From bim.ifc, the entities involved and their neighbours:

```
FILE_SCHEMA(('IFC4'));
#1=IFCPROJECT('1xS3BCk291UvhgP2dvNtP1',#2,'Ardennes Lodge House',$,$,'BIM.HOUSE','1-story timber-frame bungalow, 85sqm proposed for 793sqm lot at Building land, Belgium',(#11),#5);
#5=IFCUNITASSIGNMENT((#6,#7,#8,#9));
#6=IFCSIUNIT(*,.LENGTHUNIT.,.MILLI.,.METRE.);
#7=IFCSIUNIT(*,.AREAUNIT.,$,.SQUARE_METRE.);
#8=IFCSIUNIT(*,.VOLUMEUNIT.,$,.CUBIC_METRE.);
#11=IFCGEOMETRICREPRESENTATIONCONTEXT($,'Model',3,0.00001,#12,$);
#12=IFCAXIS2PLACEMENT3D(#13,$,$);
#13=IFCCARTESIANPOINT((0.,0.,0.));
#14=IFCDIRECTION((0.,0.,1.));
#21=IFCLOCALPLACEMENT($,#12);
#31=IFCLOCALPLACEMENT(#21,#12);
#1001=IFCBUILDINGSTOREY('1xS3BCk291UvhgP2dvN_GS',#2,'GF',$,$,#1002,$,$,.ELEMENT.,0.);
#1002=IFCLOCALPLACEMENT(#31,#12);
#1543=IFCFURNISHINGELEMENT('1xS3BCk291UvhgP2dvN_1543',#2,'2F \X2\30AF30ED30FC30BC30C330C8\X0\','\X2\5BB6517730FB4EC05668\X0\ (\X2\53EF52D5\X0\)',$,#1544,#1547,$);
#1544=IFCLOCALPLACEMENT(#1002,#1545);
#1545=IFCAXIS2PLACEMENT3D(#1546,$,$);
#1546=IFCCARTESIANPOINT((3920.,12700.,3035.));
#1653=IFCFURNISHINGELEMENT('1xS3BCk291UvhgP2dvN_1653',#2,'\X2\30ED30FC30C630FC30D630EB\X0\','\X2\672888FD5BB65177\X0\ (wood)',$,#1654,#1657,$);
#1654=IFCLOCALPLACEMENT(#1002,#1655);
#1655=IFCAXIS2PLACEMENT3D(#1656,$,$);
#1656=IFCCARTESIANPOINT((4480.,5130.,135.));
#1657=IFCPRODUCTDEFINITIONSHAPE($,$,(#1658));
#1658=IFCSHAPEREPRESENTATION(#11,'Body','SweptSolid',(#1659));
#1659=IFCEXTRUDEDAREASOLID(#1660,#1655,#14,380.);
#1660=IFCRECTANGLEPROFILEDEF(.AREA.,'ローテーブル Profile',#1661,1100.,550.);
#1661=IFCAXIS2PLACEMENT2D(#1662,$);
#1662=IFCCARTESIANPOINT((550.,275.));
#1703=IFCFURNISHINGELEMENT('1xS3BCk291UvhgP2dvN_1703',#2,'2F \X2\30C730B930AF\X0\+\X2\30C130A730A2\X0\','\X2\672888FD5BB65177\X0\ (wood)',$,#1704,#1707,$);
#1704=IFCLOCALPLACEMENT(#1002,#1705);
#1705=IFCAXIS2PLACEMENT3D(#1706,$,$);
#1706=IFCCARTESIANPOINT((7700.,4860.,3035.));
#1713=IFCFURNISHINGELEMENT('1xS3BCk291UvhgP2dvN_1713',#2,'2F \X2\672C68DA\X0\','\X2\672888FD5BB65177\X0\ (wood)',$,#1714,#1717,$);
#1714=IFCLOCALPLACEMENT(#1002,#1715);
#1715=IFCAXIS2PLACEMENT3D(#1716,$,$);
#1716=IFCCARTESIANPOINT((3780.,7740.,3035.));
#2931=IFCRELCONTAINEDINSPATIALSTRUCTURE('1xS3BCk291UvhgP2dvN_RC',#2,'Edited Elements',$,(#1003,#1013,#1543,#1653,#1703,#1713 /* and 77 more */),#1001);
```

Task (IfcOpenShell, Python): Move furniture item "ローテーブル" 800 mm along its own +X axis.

```python
import ifcopenshell
import ifcopenshell.api.geometry
import ifcopenshell.util.placement
import ifcopenshell.util.unit

model = ifcopenshell.open("bim.ifc")
unit_scale = ifcopenshell.util.unit.calculate_unit_scale(model)

item = model.by_guid("1xS3BCk291UvhgP2dvN_1653")
matrix = ifcopenshell.util.placement.get_local_placement(item.ObjectPlacement)
matrix[:3, 3] += matrix[:3, 0] * 0.8 / unit_scale
ifcopenshell.api.geometry.edit_object_placement(model, product=item, matrix=matrix, is_si=False)

print(ifcopenshell.util.placement.get_local_placement(item.ObjectPlacement).round(3) + 0.0)

model.write("bim_rev.ifc")
```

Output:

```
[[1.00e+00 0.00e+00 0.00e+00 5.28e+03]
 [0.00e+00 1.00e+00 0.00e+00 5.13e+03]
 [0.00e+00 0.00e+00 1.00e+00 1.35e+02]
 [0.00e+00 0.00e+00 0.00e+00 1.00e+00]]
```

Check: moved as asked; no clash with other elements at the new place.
